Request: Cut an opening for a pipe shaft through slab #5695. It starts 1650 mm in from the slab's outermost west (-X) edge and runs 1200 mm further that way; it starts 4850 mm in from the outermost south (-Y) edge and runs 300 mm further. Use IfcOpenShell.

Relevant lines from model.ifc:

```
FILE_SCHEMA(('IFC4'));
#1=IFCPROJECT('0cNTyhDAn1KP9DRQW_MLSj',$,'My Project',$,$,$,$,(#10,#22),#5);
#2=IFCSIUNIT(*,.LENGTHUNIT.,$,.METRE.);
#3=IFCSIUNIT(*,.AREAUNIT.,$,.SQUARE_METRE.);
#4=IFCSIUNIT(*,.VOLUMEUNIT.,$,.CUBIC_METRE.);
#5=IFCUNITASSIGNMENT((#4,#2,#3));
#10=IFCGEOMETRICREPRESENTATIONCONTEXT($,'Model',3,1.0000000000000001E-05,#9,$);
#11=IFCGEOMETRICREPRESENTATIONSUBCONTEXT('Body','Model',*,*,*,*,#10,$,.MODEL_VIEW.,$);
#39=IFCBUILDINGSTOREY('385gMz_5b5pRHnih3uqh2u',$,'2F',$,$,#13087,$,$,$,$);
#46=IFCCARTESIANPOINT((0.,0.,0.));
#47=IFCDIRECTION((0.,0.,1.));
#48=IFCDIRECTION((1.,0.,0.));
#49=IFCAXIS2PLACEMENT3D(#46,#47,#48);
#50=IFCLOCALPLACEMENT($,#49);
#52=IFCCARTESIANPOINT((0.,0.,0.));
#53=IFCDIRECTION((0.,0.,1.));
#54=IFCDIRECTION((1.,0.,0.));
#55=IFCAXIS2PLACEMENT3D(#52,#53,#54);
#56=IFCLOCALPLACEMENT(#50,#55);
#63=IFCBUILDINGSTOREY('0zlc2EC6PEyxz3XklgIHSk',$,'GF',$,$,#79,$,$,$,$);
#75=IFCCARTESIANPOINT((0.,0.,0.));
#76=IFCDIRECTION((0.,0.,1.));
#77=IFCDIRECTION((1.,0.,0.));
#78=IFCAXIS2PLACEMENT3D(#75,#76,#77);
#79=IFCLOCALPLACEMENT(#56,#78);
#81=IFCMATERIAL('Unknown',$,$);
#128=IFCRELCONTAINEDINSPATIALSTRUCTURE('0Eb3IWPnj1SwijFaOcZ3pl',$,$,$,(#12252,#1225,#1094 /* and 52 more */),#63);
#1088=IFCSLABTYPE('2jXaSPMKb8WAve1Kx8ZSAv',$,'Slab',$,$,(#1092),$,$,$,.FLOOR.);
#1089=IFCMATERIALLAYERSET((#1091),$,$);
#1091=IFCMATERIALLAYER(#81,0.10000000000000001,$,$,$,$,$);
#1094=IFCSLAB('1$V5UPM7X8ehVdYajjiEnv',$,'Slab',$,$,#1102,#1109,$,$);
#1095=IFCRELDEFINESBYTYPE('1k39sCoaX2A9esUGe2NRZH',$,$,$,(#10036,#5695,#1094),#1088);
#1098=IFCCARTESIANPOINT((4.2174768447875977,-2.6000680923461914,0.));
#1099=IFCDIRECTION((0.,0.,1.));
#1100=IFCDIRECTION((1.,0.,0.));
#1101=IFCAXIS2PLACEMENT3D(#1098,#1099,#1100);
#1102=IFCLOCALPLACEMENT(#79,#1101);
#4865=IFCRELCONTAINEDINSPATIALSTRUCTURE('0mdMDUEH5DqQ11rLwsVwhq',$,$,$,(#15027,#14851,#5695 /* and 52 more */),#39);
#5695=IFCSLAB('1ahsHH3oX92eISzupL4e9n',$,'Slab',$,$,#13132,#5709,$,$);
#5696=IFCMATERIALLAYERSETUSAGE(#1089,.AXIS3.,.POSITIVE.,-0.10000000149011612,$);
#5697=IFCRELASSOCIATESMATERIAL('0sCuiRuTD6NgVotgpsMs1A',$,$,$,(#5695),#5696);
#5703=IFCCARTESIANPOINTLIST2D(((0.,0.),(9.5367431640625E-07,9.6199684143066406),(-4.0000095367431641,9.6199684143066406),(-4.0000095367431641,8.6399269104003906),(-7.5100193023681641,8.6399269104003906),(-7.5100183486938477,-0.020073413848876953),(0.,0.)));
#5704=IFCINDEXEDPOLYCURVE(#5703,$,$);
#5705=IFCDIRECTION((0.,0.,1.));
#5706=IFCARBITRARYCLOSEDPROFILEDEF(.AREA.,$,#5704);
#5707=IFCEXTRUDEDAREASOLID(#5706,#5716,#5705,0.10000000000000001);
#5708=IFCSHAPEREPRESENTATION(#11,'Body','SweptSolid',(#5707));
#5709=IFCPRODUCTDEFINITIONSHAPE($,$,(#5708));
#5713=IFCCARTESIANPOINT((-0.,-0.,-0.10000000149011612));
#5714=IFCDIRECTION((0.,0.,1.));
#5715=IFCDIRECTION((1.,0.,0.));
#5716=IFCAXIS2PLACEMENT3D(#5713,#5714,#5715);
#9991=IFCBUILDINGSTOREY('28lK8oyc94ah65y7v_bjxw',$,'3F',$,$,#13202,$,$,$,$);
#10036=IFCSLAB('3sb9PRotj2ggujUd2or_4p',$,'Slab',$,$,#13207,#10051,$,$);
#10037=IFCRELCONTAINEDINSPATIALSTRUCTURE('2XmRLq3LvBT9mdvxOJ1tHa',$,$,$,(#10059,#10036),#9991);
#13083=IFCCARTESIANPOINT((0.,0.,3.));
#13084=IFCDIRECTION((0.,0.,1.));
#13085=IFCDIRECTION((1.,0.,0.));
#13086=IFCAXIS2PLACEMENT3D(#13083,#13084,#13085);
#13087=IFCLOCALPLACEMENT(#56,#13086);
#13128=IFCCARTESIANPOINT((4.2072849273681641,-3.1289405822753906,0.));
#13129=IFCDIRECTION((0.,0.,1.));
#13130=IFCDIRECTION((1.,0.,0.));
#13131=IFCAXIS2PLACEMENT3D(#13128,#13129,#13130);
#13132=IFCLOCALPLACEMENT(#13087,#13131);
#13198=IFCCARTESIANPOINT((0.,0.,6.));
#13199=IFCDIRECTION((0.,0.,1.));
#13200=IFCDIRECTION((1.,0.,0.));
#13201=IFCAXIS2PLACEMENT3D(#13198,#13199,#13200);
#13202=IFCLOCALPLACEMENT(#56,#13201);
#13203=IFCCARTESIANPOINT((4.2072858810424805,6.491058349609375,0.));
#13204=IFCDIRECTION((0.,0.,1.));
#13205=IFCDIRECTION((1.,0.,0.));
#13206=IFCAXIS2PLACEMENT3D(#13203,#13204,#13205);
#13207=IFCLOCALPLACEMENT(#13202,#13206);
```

```python
import numpy as np
import ifcopenshell
import ifcopenshell.api.feature
import ifcopenshell.api.geometry
import ifcopenshell.api.root
import ifcopenshell.geom
import ifcopenshell.util.placement
import ifcopenshell.util.representation
import ifcopenshell.util.shape
import ifcopenshell.util.unit

model = ifcopenshell.open("model.ifc")
unit_scale = ifcopenshell.util.unit.calculate_unit_scale(model)
settings = ifcopenshell.geom.settings()


def volume(element):
    """Net volume in cubic metres, openings subtracted."""
    shape = ifcopenshell.geom.create_shape(settings, element)
    return ifcopenshell.util.shape.get_volume(shape.geometry)


slab = model.by_guid("1ahsHH3oX92eISzupL4e9n")
before = volume(slab)

# Extent in the slab's own axes, in metres. The edges named are its -X and -Y sides.
slab_shape = ifcopenshell.geom.create_shape(settings, slab)
vertices = ifcopenshell.util.shape.get_vertices(slab_shape.geometry)
x_min, y_min, bottom = vertices.min(axis=0)
top = vertices[:, 2].max()

opening = ifcopenshell.api.root.create_entity(model, ifc_class="IfcOpeningElement", name="Pipe shaft opening", predefined_type="OPENING")
context = ifcopenshell.util.representation.get_context(model, "Model", "Body", "MODEL_VIEW")
width, depth = 1.2, 0.3
outline = [(0.0, 0.0), (width, 0.0), (width, depth), (0.0, depth), (0.0, 0.0)]
# Overshoot both faces by 50 mm so the cut is clean.
shape = ifcopenshell.api.geometry.add_slab_representation(
    model, context=context, depth=top - bottom + 0.1, polyline=outline
)
ifcopenshell.api.geometry.assign_representation(model, product=opening, representation=shape)

matrix = ifcopenshell.util.placement.get_local_placement(slab.ObjectPlacement)
matrix[:, 3] = matrix @ np.append(np.array([x_min + 1.65, y_min + 4.85, bottom - 0.05]) / unit_scale, 1.0)
ifcopenshell.api.geometry.edit_object_placement(model, product=opening, matrix=matrix, is_si=False)
ifcopenshell.api.feature.add_feature(model, feature=opening, element=slab)

after = volume(slab)

print(f"slab volume {before:.3f} -> {after:.3f} m3")

model.write("model_rev.ifc")
```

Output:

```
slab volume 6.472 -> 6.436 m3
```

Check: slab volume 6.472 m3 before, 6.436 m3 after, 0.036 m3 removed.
